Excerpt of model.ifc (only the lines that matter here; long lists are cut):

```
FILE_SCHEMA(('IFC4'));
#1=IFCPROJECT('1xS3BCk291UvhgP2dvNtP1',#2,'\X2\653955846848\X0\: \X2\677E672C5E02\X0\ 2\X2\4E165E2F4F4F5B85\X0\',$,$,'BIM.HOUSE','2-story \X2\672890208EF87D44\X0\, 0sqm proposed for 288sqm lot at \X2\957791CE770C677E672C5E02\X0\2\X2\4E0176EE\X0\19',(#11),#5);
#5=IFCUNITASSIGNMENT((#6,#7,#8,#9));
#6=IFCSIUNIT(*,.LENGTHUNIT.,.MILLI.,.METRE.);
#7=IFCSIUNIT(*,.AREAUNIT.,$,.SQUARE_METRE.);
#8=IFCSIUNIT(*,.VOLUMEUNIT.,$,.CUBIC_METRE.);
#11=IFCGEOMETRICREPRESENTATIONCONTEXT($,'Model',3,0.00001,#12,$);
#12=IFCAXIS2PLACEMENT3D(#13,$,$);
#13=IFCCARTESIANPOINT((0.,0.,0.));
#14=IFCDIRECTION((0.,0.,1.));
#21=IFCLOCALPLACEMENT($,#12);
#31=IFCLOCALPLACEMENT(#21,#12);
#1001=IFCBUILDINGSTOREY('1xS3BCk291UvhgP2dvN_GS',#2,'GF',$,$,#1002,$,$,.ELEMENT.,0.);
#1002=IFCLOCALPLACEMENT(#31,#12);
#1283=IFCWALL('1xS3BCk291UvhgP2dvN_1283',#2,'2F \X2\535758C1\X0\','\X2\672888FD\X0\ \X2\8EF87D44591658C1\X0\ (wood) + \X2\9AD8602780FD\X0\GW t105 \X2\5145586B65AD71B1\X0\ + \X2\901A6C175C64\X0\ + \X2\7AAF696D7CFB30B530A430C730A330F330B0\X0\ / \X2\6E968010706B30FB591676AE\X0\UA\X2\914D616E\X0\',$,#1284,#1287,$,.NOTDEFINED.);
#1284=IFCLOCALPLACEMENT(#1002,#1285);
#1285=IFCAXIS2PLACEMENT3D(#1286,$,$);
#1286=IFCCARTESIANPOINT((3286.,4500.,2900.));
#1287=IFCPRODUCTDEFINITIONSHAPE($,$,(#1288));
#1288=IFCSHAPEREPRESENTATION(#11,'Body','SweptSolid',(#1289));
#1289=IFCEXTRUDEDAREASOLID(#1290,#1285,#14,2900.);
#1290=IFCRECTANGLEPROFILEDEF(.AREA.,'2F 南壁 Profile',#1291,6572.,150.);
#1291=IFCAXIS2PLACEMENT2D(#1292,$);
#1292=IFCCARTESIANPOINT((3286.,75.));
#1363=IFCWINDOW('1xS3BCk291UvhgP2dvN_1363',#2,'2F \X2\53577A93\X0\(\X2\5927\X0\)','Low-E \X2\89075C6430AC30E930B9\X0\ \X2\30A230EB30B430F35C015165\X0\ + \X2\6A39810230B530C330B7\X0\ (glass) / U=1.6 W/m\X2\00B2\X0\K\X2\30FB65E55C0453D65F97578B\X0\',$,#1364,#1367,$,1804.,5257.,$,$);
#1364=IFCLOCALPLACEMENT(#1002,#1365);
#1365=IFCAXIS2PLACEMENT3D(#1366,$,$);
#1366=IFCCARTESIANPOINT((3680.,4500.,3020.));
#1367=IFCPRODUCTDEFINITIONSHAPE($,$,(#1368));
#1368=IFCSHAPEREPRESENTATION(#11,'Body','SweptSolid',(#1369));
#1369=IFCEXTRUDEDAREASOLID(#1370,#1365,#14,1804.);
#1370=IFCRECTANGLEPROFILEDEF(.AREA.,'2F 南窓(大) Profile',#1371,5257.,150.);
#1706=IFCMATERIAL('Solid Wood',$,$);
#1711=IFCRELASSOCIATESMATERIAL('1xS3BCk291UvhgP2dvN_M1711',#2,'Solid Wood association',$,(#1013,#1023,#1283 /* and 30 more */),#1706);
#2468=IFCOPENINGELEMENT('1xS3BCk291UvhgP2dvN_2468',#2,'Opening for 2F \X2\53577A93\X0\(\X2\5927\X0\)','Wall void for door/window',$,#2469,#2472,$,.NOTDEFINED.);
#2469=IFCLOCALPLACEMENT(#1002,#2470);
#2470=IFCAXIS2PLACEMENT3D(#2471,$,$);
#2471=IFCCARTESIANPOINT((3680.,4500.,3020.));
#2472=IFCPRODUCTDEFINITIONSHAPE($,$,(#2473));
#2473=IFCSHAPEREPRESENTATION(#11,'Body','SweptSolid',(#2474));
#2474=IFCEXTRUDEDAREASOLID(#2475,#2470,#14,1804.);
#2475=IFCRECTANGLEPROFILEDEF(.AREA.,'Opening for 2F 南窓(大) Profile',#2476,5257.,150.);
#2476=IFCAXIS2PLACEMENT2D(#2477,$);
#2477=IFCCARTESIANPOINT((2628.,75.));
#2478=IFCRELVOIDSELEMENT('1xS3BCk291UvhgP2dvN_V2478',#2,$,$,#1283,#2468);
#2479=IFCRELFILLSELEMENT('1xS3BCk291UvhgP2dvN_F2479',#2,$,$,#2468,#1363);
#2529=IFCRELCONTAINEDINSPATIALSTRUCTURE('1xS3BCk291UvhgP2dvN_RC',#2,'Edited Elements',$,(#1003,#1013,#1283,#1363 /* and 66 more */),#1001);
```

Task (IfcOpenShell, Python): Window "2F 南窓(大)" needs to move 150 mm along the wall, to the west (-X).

```python
import ifcopenshell
import ifcopenshell.api.geometry
import ifcopenshell.util.placement

model = ifcopenshell.open("model.ifc")

window = model.by_guid("1xS3BCk291UvhgP2dvN_1363")
opening = window.FillsVoids[0].RelatingOpeningElement
wall = opening.VoidsElements[0].RelatingBuildingElement

wall_matrix = ifcopenshell.util.placement.get_local_placement(wall.ObjectPlacement)
shift = wall_matrix[:3, 0] * -150.0
before = ifcopenshell.util.placement.get_local_placement(window.ObjectPlacement)[:3, 3].copy()

# The window is not placed relative to its opening, so move both.
for product in (opening, window):
    matrix = ifcopenshell.util.placement.get_local_placement(product.ObjectPlacement)
    matrix[:3, 3] += shift
    ifcopenshell.api.geometry.edit_object_placement(model, product=product, matrix=matrix, is_si=False)

after = ifcopenshell.util.placement.get_local_placement(window.ObjectPlacement)[:3, 3]
print("window moved by", (after - before).round(3) + 0.0)

model.write("model_edited.ifc")
```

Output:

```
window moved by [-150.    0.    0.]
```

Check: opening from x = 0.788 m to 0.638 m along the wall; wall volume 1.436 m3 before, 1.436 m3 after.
